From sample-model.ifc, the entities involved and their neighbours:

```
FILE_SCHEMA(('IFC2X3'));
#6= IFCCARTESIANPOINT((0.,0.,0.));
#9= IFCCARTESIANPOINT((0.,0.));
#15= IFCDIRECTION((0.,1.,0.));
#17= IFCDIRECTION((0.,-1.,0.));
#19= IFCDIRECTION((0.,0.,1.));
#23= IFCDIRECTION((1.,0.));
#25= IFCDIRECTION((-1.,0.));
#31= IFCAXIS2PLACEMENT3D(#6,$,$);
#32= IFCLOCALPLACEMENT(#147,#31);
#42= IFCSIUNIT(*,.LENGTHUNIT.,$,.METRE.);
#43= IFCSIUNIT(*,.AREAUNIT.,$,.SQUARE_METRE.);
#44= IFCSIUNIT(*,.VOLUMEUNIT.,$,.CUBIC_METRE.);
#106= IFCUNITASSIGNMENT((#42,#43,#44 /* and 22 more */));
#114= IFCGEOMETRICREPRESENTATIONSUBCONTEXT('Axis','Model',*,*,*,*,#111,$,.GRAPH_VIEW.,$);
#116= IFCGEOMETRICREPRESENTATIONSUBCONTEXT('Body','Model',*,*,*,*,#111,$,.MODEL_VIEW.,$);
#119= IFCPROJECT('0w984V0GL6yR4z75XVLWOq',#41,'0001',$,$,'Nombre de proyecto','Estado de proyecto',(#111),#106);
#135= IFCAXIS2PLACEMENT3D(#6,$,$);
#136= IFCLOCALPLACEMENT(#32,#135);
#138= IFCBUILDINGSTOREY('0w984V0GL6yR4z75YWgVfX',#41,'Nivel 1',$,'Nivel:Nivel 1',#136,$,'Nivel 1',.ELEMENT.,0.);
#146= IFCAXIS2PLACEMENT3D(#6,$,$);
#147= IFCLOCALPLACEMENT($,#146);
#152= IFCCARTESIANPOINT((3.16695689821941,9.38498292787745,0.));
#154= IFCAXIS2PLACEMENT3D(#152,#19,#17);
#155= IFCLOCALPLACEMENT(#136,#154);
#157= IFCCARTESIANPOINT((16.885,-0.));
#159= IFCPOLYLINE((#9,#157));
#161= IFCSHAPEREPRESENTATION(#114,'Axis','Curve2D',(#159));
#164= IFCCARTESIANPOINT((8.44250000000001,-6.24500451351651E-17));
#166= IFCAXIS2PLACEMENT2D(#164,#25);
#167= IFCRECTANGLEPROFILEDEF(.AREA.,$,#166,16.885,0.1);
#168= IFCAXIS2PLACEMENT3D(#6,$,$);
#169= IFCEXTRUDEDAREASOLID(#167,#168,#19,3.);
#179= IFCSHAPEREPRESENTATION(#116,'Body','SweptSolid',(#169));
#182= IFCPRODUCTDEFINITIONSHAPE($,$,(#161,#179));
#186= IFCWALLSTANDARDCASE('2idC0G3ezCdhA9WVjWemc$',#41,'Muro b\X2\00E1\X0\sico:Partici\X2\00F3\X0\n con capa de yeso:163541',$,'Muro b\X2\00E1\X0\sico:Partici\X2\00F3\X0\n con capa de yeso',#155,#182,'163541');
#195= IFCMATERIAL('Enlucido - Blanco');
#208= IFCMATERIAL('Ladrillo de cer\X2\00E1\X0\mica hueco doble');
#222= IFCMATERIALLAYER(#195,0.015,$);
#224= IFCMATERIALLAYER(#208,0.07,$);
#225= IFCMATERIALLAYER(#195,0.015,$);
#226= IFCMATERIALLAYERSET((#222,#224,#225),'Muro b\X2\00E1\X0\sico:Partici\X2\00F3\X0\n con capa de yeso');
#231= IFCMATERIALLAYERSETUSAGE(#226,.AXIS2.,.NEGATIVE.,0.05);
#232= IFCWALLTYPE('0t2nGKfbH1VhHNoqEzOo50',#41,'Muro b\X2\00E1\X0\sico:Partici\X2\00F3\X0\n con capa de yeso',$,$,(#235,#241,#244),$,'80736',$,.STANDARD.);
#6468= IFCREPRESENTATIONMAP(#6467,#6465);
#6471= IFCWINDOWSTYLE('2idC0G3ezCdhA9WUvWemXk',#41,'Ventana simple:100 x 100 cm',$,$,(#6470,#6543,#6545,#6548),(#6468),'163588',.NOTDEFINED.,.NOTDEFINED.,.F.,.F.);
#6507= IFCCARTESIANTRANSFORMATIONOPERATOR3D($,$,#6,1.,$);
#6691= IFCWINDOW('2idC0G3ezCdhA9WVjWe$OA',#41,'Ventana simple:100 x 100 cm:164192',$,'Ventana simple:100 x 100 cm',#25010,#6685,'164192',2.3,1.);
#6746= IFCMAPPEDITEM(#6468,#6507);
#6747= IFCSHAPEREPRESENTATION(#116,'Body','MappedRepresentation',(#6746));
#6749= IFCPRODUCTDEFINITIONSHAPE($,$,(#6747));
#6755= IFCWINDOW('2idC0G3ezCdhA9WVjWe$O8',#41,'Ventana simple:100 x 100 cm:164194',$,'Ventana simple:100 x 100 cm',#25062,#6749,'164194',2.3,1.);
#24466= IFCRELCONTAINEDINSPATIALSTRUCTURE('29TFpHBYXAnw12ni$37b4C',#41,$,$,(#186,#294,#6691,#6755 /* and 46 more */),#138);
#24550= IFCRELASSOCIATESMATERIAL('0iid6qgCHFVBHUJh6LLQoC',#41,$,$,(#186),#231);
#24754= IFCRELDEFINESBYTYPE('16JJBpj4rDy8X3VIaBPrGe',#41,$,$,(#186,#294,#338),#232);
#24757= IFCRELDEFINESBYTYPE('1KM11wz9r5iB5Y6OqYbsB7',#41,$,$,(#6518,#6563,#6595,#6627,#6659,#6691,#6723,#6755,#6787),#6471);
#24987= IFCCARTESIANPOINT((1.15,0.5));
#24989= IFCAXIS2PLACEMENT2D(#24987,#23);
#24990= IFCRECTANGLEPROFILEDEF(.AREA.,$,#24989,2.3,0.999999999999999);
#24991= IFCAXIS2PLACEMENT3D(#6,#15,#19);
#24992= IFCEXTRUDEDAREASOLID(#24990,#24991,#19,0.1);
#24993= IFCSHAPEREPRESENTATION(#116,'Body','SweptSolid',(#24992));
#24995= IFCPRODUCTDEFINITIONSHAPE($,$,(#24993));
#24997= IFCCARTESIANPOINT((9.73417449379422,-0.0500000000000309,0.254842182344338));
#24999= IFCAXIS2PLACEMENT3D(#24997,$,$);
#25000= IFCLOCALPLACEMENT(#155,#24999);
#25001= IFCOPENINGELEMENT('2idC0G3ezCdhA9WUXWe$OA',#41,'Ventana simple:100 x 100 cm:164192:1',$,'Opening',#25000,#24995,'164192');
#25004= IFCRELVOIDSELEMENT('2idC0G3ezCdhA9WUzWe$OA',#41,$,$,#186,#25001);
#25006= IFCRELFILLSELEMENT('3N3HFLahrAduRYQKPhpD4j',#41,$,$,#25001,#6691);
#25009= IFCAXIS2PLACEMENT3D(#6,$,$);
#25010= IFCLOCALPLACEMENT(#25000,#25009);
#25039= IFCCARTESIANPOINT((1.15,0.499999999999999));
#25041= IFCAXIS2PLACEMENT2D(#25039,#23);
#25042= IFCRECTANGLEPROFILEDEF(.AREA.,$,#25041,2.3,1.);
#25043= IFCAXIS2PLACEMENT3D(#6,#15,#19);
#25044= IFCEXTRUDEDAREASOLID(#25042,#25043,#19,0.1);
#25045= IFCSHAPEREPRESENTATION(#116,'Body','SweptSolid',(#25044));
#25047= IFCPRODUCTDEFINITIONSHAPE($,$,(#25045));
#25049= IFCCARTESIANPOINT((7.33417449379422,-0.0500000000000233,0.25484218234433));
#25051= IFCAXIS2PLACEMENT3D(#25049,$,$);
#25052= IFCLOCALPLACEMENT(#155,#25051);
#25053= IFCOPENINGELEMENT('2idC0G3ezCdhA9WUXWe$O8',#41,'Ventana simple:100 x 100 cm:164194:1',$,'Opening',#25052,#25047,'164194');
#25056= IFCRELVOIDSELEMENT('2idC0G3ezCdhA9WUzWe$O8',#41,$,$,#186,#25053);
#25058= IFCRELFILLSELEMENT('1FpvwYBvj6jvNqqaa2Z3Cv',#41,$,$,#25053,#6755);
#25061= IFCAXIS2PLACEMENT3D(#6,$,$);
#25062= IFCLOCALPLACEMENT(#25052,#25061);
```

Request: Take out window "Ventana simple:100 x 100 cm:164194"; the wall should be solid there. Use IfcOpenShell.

```python
import ifcopenshell
import ifcopenshell.api.feature
import ifcopenshell.api.root
import ifcopenshell.geom
import ifcopenshell.util.shape

model = ifcopenshell.open("sample-model.ifc")
settings = ifcopenshell.geom.settings()


def volume(element):
    """Net volume in cubic metres, openings subtracted."""
    shape = ifcopenshell.geom.create_shape(settings, element)
    return ifcopenshell.util.shape.get_volume(shape.geometry)


window = model.by_guid("2idC0G3ezCdhA9WVjWe$O8")
opening = window.FillsVoids[0].RelatingOpeningElement
wall = opening.VoidsElements[0].RelatingBuildingElement
before = volume(wall)

ifcopenshell.api.root.remove_product(model, product=window)
ifcopenshell.api.feature.remove_feature(model, feature=opening)

after = volume(wall)

print(f"wall volume {before:.3f} -> {after:.3f} m3")

model.write("sample-model_rev.ifc")
```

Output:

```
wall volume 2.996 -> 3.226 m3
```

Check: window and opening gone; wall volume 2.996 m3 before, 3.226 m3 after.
